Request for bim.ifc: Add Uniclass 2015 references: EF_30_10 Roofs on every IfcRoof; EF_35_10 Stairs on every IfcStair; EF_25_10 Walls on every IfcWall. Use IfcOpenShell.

First a look at what the model holds.

```python
import ifcopenshell

model = ifcopenshell.open("bim.ifc")
print(model.schema)
print("classifications:", [c.Name for c in model.by_type("IfcClassification")])
for ifc_class in ("IfcDoor", "IfcRoof", "IfcStair", "IfcWall", "IfcWindow"):
    print(ifc_class, len(model.by_type(ifc_class)))
```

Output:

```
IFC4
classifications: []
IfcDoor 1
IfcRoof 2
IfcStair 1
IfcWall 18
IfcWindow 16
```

```python
import ifcopenshell
import ifcopenshell.api.classification

model = ifcopenshell.open("bim.ifc")

system = ifcopenshell.api.classification.add_classification(model, classification="Uniclass 2015")

codes = {
    "IfcRoof": ("EF_30_10", "Roofs"),
    "IfcStair": ("EF_35_10", "Stairs"),
    "IfcWall": ("EF_25_10", "Walls"),
}
for ifc_class, (code, name) in codes.items():
    products = model.by_type(ifc_class)
    ifcopenshell.api.classification.add_reference(
        model, products=products, classification=system, identification=code, name=name
    )
    print(code, len(products))

model.write("bim_edited.ifc")
```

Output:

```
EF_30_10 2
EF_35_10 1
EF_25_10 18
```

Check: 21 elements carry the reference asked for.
